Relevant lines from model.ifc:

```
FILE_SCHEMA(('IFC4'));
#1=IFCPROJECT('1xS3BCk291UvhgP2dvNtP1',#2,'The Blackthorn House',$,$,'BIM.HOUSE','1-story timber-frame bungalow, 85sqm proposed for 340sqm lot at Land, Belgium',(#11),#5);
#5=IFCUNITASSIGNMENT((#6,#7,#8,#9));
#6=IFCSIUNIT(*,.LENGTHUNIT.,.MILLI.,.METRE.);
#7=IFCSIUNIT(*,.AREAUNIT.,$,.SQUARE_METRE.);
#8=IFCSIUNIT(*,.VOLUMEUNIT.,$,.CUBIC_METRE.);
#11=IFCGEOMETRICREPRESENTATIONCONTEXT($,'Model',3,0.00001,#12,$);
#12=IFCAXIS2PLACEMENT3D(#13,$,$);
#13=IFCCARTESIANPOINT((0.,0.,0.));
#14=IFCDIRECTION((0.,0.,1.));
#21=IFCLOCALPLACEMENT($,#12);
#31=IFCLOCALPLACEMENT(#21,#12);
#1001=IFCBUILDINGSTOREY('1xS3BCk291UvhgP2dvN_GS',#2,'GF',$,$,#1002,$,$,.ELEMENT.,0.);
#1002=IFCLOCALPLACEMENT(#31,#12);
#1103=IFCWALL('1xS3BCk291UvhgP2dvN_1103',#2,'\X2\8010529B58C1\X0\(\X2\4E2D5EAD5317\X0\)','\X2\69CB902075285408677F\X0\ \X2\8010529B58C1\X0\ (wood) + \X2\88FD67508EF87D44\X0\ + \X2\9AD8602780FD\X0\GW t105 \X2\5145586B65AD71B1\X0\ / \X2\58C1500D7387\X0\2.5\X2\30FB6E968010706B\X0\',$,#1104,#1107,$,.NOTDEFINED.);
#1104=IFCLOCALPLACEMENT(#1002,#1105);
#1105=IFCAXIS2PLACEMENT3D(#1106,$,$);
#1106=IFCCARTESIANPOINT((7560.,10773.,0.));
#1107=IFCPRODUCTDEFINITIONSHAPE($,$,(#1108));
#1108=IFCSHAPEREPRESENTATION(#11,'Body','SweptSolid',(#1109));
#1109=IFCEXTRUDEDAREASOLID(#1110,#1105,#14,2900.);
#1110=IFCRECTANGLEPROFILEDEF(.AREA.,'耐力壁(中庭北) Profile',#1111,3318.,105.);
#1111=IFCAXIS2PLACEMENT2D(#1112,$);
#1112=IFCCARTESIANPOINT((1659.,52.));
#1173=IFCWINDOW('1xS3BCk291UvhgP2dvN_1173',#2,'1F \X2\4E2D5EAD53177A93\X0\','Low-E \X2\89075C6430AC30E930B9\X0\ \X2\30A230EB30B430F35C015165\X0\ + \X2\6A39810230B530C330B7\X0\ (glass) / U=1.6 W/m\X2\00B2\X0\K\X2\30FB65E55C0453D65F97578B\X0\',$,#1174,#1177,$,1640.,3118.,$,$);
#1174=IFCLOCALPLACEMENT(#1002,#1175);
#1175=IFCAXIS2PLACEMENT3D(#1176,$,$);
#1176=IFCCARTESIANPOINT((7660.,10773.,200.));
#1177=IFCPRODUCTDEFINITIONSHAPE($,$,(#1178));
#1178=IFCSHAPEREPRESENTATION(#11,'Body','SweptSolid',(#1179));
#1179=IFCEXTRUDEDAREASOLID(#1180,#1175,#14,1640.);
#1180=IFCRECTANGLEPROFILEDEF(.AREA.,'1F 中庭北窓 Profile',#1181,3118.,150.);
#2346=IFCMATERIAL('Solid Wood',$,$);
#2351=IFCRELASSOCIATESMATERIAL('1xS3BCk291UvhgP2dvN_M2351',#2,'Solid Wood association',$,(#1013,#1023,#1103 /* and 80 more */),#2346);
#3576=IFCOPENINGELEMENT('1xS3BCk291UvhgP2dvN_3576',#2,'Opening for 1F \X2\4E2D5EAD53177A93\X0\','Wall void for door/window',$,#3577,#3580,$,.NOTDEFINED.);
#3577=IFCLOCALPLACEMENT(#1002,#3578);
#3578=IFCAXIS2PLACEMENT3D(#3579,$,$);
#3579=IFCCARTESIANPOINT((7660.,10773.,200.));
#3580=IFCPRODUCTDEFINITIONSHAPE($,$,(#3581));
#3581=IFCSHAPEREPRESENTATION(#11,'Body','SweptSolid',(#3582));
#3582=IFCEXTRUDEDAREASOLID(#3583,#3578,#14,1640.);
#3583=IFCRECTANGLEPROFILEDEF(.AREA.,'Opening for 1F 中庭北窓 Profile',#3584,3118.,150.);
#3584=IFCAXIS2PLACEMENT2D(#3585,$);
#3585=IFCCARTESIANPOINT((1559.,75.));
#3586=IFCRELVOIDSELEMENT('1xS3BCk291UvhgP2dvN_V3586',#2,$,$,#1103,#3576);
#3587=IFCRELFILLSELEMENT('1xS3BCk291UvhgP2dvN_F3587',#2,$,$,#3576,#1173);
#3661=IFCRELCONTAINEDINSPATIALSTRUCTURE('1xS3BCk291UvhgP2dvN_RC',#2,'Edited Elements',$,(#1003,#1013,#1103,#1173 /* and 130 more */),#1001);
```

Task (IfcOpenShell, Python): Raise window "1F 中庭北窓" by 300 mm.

```python
import numpy as np
import ifcopenshell
import ifcopenshell.api.geometry
import ifcopenshell.util.placement
import ifcopenshell.util.unit

model = ifcopenshell.open("model.ifc")
unit_scale = ifcopenshell.util.unit.calculate_unit_scale(model)

window = model.by_guid("1xS3BCk291UvhgP2dvN_1173")
opening = window.FillsVoids[0].RelatingOpeningElement
dz = 300.0

shift = np.array([0.0, 0.0, dz])
# The window is not placed relative to its opening, so move both.
for product in (opening, window):
    matrix = ifcopenshell.util.placement.get_local_placement(product.ObjectPlacement)
    matrix[:3, 3] += shift
    ifcopenshell.api.geometry.edit_object_placement(model, product=product, matrix=matrix, is_si=False)

print(f"moved by {dz * unit_scale:+.3f} m")

model.write("model_updated.ifc")
```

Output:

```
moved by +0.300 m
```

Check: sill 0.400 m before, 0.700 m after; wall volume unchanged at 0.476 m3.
